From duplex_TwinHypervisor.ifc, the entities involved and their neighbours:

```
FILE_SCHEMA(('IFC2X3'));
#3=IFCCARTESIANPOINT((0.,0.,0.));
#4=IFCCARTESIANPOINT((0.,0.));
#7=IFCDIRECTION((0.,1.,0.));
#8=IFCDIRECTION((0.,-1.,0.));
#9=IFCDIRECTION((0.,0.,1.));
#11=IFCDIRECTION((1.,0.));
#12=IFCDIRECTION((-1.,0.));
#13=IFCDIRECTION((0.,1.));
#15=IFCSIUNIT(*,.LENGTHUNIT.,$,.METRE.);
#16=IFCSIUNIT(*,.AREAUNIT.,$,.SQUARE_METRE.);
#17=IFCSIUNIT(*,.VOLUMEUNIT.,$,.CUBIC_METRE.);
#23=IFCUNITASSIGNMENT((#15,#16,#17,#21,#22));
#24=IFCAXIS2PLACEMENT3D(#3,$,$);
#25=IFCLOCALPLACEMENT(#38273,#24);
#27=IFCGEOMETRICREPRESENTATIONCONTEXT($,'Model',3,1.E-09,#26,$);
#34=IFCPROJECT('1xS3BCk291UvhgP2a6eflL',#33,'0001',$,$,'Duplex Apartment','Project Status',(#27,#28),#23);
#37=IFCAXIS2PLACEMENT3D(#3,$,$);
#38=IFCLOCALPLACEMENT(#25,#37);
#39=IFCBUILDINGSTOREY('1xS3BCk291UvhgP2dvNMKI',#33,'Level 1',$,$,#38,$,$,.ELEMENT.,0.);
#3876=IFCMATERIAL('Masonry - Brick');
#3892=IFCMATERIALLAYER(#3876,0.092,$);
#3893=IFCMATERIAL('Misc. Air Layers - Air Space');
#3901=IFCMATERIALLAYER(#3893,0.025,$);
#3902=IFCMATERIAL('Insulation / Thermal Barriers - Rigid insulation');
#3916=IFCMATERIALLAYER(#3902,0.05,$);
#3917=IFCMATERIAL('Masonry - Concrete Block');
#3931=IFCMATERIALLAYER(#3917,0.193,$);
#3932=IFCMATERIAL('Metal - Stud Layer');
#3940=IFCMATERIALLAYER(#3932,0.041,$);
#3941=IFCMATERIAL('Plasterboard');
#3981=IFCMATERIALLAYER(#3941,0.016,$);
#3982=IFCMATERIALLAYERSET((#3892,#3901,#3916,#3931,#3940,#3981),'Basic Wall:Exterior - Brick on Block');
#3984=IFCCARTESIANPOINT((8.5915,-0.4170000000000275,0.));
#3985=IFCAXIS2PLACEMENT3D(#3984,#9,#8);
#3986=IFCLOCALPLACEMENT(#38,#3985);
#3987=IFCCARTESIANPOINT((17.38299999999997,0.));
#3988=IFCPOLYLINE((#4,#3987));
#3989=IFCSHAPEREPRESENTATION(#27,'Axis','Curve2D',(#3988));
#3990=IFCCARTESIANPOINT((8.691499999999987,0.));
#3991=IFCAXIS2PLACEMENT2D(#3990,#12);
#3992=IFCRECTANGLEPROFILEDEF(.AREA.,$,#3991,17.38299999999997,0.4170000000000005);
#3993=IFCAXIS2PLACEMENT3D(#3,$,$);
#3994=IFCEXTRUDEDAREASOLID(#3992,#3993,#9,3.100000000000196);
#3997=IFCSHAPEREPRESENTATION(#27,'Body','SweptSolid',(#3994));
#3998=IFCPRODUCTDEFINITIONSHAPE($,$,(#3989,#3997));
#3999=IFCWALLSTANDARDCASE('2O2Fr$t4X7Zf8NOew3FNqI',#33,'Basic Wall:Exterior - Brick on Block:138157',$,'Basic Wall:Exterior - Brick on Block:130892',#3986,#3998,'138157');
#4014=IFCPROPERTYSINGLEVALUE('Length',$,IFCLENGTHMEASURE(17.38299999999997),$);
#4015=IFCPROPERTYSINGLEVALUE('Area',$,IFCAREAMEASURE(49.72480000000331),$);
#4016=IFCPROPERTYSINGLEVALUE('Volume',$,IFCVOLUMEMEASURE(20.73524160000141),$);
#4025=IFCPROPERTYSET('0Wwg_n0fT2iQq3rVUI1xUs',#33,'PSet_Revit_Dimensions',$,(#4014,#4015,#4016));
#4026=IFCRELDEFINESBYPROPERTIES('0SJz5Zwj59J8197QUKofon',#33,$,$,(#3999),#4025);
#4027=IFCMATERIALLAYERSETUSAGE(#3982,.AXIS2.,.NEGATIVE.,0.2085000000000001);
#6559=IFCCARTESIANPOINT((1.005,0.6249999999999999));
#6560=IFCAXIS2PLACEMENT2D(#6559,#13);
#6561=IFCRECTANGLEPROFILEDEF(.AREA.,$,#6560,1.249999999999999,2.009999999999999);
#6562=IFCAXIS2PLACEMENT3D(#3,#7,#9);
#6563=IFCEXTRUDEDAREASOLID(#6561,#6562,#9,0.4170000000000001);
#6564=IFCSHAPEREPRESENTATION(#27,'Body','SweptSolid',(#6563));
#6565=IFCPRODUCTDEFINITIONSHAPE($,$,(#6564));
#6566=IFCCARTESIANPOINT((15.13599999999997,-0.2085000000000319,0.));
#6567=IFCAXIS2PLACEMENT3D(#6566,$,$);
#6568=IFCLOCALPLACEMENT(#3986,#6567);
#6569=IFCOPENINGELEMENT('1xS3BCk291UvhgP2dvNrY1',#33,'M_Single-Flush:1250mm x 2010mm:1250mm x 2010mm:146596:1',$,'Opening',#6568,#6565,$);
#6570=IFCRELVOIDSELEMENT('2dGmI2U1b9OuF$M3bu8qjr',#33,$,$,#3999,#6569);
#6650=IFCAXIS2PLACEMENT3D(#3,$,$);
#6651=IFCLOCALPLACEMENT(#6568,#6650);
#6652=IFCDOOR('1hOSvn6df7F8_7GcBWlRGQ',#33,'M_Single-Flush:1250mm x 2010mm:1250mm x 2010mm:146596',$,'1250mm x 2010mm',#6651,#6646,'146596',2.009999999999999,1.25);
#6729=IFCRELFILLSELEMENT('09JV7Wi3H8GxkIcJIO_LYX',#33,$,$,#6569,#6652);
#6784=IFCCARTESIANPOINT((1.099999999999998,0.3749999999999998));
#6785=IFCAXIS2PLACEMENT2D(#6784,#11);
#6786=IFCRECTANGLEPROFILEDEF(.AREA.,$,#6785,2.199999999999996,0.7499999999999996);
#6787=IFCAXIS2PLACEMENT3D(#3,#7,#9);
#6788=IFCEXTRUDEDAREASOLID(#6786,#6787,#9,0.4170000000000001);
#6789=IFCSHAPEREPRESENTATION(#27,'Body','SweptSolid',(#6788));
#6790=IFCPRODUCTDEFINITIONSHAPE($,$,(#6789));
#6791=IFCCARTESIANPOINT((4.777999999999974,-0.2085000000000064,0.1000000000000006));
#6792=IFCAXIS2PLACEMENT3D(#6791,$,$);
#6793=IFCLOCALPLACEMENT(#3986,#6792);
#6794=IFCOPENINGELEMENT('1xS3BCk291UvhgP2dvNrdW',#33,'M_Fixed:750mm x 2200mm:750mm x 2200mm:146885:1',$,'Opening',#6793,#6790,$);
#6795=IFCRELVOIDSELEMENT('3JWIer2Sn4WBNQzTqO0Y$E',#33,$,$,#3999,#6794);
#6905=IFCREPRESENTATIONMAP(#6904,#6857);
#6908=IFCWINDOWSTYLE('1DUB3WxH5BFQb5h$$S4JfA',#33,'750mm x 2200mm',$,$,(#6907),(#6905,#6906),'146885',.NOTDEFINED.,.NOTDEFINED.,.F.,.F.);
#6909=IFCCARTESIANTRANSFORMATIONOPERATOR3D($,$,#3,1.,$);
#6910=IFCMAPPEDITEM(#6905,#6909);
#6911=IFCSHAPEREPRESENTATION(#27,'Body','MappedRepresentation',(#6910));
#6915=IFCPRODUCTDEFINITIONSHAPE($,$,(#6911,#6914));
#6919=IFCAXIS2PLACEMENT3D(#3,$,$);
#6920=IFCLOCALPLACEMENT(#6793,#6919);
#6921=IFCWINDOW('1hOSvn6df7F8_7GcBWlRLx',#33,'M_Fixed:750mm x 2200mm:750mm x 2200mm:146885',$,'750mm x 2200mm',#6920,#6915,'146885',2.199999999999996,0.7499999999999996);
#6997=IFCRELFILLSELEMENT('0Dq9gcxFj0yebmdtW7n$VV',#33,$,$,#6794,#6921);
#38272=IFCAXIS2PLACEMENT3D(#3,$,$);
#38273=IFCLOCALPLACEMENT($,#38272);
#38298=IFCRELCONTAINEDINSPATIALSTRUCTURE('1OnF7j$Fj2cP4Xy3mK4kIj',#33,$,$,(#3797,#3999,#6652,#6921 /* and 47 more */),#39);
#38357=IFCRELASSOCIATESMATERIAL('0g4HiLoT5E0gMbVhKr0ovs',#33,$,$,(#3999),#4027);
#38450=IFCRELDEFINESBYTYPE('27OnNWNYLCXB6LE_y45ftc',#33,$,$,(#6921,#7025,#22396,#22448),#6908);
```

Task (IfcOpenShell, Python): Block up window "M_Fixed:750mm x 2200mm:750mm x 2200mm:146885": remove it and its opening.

```python
import ifcopenshell
import ifcopenshell.api.feature
import ifcopenshell.api.pset
import ifcopenshell.api.root
import ifcopenshell.geom
import ifcopenshell.util.element
import ifcopenshell.util.shape
import ifcopenshell.util.unit

model = ifcopenshell.open("duplex_TwinHypervisor.ifc")
area_scale = ifcopenshell.util.unit.calculate_unit_scale(model, "AREAUNIT")
volume_scale = ifcopenshell.util.unit.calculate_unit_scale(model, "VOLUMEUNIT")
settings = ifcopenshell.geom.settings()


def volume(element):
    """Net volume in cubic metres, openings subtracted."""
    shape = ifcopenshell.geom.create_shape(settings, element)
    return ifcopenshell.util.shape.get_volume(shape.geometry)


window = model.by_id(6921)
opening = window.FillsVoids[0].RelatingOpeningElement
wall = opening.VoidsElements[0].RelatingBuildingElement
before = volume(wall)

ifcopenshell.api.root.remove_product(model, product=window)
ifcopenshell.api.feature.remove_feature(model, feature=opening)

after = volume(wall)
thickness = 0.417  # wall thickness in metres

# Update the wall's stored quantities.
pset = model.by_id(ifcopenshell.util.element.get_pset(wall, "PSet_Revit_Dimensions", should_inherit=False)["id"])
ifcopenshell.api.pset.edit_pset(model, pset=pset, properties={
    "Area": model.create_entity("IfcAreaMeasure", after / thickness / area_scale),
    "Volume": model.create_entity("IfcVolumeMeasure", after / volume_scale),
})

print(f"wall volume {before:.3f} -> {after:.3f} m3")

model.write("duplex_TwinHypervisor_updated.ifc")
```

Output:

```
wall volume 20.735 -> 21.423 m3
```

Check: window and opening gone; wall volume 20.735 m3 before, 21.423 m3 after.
